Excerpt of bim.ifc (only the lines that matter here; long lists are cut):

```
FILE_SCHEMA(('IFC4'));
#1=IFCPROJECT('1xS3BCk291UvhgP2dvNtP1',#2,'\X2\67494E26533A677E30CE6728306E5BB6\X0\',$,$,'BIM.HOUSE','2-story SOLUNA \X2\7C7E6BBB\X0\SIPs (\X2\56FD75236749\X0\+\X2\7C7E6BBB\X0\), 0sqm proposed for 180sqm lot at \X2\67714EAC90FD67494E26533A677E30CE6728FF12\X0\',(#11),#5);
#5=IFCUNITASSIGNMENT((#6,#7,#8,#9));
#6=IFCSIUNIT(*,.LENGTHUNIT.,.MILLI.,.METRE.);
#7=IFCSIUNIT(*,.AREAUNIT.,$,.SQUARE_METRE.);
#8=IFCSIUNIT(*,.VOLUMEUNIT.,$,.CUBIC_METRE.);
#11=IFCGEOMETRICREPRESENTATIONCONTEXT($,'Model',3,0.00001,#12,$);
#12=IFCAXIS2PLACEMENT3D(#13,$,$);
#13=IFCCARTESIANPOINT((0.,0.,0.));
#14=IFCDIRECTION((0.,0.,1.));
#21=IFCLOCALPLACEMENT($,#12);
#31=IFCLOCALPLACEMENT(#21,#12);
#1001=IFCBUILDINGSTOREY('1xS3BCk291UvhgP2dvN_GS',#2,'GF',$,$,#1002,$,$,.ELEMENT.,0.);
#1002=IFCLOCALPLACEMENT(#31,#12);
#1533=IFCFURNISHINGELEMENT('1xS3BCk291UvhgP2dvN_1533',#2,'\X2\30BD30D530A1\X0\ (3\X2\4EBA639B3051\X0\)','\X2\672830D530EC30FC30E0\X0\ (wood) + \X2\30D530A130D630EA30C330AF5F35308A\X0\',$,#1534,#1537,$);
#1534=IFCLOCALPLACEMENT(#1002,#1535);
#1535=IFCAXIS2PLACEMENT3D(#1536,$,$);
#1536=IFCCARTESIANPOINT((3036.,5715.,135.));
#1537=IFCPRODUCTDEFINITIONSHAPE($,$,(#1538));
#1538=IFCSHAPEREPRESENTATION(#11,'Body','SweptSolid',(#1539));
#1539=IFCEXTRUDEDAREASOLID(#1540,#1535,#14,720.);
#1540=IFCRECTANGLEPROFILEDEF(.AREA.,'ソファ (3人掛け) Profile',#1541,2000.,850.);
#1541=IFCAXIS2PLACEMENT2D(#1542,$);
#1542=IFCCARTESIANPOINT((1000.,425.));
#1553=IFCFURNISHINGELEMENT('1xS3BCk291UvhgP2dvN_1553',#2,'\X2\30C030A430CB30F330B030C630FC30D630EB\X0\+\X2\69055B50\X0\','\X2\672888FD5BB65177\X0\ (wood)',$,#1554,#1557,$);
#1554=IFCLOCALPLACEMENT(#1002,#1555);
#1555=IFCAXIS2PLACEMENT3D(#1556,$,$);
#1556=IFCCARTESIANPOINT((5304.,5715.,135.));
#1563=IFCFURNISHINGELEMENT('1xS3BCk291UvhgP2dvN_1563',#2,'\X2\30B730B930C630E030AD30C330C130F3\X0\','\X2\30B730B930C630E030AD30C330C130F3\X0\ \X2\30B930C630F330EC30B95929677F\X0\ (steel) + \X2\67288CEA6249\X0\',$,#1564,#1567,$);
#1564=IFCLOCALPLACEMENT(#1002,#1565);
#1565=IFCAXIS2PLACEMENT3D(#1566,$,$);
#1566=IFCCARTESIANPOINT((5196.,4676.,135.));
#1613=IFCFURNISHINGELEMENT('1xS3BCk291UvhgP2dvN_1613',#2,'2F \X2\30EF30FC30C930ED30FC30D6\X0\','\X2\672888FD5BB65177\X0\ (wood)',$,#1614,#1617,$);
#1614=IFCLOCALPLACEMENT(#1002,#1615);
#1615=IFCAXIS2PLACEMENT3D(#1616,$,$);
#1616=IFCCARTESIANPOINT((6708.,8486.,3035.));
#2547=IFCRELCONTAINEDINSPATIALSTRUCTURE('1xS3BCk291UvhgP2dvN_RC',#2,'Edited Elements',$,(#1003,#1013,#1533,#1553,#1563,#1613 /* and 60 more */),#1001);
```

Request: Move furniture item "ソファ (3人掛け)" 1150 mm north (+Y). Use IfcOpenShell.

```python
import ifcopenshell
import ifcopenshell.api.geometry
import ifcopenshell.util.placement

model = ifcopenshell.open("bim.ifc")

item = model.by_id(1533)
matrix = ifcopenshell.util.placement.get_local_placement(item.ObjectPlacement)
matrix[1, 3] += 1150.0
ifcopenshell.api.geometry.edit_object_placement(model, product=item, matrix=matrix, is_si=False)

print(ifcopenshell.util.placement.get_local_placement(item.ObjectPlacement).round(3) + 0.0)

model.write("bim_rev.ifc")
```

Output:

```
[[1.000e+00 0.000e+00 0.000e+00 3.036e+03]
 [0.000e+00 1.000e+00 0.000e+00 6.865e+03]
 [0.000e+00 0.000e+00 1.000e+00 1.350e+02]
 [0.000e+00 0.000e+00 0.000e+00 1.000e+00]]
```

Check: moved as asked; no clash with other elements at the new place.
